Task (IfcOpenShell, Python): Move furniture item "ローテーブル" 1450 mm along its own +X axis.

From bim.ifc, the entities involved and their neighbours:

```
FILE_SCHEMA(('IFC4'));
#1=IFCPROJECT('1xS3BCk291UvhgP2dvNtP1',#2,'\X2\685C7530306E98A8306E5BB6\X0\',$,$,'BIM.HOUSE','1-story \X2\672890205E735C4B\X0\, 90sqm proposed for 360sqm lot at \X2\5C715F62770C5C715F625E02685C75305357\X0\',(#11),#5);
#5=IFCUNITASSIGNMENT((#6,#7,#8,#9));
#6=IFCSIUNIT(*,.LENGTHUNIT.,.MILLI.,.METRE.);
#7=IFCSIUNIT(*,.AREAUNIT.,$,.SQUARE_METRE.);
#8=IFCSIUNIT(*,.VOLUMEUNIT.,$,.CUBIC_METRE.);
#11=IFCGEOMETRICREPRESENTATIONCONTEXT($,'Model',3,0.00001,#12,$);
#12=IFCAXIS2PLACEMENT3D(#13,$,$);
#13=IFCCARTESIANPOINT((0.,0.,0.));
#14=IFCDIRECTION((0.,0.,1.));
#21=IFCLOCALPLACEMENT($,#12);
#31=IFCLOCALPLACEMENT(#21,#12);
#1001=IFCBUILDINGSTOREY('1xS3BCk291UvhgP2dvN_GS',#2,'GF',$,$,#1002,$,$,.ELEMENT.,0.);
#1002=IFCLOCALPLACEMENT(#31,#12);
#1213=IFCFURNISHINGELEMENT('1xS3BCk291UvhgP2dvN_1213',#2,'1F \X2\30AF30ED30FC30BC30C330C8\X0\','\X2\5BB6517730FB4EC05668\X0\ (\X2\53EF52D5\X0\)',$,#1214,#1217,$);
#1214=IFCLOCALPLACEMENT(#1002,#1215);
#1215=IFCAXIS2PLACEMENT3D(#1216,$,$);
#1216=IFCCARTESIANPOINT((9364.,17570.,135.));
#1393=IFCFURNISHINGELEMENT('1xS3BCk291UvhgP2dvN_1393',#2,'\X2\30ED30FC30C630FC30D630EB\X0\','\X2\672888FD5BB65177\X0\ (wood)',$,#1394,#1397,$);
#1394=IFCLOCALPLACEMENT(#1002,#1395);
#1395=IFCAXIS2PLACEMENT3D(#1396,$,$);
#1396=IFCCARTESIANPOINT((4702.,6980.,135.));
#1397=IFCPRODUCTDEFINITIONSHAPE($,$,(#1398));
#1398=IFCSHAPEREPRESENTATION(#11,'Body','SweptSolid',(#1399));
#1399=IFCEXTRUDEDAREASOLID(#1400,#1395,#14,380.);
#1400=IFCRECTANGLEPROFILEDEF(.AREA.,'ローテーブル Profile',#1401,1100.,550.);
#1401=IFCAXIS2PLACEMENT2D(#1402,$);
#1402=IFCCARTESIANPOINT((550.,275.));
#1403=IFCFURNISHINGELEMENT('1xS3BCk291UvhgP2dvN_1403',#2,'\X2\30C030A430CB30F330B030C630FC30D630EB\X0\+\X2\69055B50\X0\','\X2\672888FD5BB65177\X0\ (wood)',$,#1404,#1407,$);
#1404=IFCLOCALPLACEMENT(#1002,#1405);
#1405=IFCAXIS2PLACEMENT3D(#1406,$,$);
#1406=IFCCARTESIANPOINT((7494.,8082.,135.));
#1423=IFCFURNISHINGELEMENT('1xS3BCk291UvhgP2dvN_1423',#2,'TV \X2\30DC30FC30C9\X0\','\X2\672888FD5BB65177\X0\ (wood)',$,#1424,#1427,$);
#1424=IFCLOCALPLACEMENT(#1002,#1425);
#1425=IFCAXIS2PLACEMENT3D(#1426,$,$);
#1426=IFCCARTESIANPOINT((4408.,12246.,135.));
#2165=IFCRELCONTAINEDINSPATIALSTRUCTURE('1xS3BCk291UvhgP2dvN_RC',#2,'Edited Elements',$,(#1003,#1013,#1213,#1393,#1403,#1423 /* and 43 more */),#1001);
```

```python
import ifcopenshell
import ifcopenshell.api.geometry
import ifcopenshell.util.placement
import ifcopenshell.util.unit

model = ifcopenshell.open("bim.ifc")
unit_scale = ifcopenshell.util.unit.calculate_unit_scale(model)

item = model.by_guid("1xS3BCk291UvhgP2dvN_1393")
matrix = ifcopenshell.util.placement.get_local_placement(item.ObjectPlacement)
matrix[:3, 3] += matrix[:3, 0] * 1.45 / unit_scale
ifcopenshell.api.geometry.edit_object_placement(model, product=item, matrix=matrix, is_si=False)

print(ifcopenshell.util.placement.get_local_placement(item.ObjectPlacement).round(3) + 0.0)

model.write("bim-out.ifc")
```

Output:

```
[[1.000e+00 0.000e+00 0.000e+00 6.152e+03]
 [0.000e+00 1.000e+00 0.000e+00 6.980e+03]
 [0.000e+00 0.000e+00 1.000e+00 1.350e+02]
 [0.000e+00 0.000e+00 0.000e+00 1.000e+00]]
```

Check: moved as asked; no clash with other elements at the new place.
